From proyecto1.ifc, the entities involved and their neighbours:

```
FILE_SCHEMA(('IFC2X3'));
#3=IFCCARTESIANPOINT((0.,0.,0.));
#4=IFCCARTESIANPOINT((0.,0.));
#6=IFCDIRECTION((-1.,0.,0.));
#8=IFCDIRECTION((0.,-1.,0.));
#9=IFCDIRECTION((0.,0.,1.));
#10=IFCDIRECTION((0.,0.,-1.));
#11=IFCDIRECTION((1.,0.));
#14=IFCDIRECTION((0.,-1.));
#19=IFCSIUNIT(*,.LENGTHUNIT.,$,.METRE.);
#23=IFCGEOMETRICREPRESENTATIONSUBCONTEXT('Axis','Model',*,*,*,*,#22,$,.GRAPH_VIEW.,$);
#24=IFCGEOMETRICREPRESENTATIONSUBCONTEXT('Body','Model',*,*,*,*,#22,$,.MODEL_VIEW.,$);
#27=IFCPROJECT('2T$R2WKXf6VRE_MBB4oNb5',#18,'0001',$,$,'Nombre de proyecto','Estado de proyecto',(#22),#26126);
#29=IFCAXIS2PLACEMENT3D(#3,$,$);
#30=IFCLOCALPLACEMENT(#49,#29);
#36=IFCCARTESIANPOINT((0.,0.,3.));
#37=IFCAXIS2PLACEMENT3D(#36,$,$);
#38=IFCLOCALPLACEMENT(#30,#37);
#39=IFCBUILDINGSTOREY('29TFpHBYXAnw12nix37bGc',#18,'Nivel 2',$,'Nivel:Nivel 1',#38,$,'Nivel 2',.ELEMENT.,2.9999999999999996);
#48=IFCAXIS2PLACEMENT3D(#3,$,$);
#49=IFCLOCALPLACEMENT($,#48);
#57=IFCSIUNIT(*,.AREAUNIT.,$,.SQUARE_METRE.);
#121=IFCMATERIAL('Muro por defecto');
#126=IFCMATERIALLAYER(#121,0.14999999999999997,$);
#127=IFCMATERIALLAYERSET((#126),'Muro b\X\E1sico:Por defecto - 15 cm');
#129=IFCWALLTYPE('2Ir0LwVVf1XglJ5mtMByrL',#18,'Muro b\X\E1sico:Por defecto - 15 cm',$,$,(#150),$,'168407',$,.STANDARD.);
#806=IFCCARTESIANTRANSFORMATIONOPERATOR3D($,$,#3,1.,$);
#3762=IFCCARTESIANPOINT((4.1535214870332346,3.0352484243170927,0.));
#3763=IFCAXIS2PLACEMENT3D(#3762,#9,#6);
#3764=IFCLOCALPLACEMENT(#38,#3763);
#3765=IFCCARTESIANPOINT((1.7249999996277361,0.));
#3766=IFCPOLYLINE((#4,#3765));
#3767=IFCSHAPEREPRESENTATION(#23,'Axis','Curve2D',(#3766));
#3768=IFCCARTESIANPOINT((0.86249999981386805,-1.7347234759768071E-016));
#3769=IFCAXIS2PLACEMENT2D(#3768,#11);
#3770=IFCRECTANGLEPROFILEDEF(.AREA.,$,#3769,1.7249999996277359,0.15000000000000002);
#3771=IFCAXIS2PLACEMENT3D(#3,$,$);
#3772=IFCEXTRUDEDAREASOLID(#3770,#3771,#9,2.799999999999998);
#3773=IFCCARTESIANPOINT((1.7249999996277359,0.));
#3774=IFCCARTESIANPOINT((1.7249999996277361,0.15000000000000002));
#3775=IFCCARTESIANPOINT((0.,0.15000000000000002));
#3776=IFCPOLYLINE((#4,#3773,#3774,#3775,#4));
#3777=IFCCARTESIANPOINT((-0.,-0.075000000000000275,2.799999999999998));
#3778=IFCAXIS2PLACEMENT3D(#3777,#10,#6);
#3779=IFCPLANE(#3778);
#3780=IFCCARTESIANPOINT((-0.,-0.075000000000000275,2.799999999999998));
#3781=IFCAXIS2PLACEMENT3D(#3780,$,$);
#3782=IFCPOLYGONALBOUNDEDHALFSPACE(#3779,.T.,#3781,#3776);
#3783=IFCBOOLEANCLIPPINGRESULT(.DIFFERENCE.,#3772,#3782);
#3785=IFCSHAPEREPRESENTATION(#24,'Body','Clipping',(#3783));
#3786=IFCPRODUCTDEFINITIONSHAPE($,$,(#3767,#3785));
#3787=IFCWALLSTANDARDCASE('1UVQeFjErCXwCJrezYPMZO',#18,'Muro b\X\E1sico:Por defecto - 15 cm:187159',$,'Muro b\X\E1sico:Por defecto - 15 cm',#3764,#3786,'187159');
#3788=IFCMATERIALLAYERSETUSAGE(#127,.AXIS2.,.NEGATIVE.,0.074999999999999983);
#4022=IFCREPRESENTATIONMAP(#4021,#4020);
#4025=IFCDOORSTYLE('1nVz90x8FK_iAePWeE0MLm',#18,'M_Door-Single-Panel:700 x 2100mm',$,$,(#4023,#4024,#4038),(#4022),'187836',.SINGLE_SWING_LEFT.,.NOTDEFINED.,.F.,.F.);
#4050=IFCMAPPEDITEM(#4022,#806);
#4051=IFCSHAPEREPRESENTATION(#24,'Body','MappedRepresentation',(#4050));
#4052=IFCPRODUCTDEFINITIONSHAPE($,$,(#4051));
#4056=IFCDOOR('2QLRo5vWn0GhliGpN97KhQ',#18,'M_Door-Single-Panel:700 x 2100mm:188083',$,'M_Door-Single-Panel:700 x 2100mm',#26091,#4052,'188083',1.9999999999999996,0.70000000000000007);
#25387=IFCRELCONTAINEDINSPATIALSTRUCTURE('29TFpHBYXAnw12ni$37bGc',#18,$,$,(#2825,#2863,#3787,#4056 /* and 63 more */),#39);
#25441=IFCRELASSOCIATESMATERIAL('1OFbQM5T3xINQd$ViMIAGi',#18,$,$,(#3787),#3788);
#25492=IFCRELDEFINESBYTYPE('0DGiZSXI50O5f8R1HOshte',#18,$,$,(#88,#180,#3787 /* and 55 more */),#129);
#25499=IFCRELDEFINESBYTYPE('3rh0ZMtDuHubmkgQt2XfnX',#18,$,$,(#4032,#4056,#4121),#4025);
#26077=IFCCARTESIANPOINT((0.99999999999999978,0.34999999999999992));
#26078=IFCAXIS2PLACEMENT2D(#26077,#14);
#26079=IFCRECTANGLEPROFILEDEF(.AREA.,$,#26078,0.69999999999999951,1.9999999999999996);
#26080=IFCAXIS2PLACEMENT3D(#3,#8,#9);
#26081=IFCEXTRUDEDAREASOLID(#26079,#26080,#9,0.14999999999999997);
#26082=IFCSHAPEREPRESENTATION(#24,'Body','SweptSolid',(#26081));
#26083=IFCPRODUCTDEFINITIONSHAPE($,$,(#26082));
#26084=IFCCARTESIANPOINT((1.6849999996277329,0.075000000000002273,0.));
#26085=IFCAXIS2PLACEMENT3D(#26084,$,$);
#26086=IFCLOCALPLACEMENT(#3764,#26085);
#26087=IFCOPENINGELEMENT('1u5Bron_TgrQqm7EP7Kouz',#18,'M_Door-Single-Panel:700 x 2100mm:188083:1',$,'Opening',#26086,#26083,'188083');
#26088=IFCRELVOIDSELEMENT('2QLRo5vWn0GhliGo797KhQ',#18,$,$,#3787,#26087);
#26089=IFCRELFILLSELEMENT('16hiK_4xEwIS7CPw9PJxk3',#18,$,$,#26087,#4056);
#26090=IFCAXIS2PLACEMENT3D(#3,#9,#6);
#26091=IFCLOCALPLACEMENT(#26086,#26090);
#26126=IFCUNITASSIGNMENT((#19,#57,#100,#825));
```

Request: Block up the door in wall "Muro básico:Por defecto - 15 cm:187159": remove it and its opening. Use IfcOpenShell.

```python
import ifcopenshell
import ifcopenshell.api.feature
import ifcopenshell.api.root
import ifcopenshell.geom
import ifcopenshell.util.shape

model = ifcopenshell.open("proyecto1.ifc")
settings = ifcopenshell.geom.settings()


def volume(element):
    """Net volume in cubic metres, openings subtracted."""
    shape = ifcopenshell.geom.create_shape(settings, element)
    return ifcopenshell.util.shape.get_volume(shape.geometry)


door = model.by_guid("2QLRo5vWn0GhliGpN97KhQ")
opening = door.FillsVoids[0].RelatingOpeningElement
wall = opening.VoidsElements[0].RelatingBuildingElement
before = volume(wall)

ifcopenshell.api.root.remove_product(model, product=door)
ifcopenshell.api.feature.remove_feature(model, feature=opening)

after = volume(wall)

print(f"wall volume {before:.3f} -> {after:.3f} m3")

model.write("proyecto1_edited.ifc")
```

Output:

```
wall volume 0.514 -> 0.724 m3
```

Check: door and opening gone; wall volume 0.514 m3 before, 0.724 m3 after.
